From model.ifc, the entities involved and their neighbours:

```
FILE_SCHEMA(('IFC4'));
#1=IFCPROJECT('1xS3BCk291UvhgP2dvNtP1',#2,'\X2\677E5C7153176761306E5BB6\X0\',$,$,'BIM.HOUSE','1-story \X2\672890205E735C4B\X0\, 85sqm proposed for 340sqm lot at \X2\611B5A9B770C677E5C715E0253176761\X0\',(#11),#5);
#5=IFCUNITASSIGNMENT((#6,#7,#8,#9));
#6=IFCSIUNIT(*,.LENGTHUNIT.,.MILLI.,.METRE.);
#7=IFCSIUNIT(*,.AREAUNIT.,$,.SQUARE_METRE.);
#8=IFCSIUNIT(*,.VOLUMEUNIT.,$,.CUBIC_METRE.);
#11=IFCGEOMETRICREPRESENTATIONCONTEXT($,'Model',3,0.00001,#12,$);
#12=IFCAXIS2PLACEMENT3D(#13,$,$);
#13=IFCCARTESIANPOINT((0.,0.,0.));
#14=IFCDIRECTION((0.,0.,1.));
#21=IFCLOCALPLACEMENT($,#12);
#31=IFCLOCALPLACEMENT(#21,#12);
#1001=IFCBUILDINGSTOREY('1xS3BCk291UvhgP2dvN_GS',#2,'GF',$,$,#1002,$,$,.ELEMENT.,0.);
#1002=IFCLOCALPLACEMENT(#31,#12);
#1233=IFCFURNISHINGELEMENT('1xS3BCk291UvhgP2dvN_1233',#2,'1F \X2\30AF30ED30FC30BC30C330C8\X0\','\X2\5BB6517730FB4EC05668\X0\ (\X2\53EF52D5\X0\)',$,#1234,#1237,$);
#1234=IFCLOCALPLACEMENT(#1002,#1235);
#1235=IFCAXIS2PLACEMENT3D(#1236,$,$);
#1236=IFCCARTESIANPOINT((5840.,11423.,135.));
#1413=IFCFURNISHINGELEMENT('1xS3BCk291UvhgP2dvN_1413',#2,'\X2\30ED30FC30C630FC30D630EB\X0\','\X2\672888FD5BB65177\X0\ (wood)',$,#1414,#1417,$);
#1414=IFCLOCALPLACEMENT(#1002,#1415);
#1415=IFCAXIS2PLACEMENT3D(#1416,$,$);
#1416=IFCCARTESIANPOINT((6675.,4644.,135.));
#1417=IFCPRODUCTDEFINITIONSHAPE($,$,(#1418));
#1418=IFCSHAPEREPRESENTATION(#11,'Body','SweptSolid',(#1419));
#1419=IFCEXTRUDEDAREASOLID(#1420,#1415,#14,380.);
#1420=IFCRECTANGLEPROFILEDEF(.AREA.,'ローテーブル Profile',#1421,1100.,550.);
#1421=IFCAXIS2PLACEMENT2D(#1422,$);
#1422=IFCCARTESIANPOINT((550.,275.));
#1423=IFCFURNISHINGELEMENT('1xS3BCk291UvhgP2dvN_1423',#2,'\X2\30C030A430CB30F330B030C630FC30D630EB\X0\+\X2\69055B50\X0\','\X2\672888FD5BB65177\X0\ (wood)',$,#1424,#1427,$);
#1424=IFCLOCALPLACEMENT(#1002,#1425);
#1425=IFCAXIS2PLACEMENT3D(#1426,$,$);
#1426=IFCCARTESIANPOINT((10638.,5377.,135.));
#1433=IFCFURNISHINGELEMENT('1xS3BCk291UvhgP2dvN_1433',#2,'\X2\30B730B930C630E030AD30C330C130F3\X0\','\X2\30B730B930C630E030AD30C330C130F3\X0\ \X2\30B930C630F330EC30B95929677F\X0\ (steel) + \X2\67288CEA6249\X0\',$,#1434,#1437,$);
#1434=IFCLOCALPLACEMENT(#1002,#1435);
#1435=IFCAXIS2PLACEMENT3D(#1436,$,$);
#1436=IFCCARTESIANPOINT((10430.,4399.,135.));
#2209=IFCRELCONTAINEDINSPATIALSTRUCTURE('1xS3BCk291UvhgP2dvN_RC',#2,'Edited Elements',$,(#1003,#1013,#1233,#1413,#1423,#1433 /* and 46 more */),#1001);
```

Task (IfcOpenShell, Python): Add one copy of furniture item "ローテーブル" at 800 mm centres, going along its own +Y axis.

```python
import ifcopenshell
import ifcopenshell.api.geometry
import ifcopenshell.api.root
import ifcopenshell.util.element
import ifcopenshell.util.placement
import ifcopenshell.util.unit

model = ifcopenshell.open("model.ifc")
unit_scale = ifcopenshell.util.unit.calculate_unit_scale(model)


def reuse_history(source, copy):
    """copy_class also copies each property set's owner history, people and application; keep the originals."""
    for rel in copy.IsDefinedBy:
        if rel.is_a("IfcRelDefinesByProperties") and (history := rel.RelatingPropertyDefinition.OwnerHistory):
            rel.RelatingPropertyDefinition.OwnerHistory = source.OwnerHistory
            ifcopenshell.util.element.remove_deep2(model, history)


source = model.by_guid("1xS3BCk291UvhgP2dvN_1413")
base = ifcopenshell.util.placement.get_local_placement(source.ObjectPlacement)
step = base[:3, 1] * 0.8 / unit_scale

for i in range(1, 2):
    copy = ifcopenshell.api.root.copy_class(model, product=source)
    copy.Representation = ifcopenshell.util.element.copy_deep(
        model, source.Representation, exclude=["IfcGeometricRepresentationContext", "IfcRepresentationMap"]
    )
    reuse_history(source, copy)
    matrix = base.copy()
    matrix[:3, 3] += i * step
    print("added at", matrix[:3, 3].round(3) + 0.0)
    ifcopenshell.api.geometry.edit_object_placement(model, product=copy, matrix=matrix, is_si=False)

model.write("model-out.ifc")
```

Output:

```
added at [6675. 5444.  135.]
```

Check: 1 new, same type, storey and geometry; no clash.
